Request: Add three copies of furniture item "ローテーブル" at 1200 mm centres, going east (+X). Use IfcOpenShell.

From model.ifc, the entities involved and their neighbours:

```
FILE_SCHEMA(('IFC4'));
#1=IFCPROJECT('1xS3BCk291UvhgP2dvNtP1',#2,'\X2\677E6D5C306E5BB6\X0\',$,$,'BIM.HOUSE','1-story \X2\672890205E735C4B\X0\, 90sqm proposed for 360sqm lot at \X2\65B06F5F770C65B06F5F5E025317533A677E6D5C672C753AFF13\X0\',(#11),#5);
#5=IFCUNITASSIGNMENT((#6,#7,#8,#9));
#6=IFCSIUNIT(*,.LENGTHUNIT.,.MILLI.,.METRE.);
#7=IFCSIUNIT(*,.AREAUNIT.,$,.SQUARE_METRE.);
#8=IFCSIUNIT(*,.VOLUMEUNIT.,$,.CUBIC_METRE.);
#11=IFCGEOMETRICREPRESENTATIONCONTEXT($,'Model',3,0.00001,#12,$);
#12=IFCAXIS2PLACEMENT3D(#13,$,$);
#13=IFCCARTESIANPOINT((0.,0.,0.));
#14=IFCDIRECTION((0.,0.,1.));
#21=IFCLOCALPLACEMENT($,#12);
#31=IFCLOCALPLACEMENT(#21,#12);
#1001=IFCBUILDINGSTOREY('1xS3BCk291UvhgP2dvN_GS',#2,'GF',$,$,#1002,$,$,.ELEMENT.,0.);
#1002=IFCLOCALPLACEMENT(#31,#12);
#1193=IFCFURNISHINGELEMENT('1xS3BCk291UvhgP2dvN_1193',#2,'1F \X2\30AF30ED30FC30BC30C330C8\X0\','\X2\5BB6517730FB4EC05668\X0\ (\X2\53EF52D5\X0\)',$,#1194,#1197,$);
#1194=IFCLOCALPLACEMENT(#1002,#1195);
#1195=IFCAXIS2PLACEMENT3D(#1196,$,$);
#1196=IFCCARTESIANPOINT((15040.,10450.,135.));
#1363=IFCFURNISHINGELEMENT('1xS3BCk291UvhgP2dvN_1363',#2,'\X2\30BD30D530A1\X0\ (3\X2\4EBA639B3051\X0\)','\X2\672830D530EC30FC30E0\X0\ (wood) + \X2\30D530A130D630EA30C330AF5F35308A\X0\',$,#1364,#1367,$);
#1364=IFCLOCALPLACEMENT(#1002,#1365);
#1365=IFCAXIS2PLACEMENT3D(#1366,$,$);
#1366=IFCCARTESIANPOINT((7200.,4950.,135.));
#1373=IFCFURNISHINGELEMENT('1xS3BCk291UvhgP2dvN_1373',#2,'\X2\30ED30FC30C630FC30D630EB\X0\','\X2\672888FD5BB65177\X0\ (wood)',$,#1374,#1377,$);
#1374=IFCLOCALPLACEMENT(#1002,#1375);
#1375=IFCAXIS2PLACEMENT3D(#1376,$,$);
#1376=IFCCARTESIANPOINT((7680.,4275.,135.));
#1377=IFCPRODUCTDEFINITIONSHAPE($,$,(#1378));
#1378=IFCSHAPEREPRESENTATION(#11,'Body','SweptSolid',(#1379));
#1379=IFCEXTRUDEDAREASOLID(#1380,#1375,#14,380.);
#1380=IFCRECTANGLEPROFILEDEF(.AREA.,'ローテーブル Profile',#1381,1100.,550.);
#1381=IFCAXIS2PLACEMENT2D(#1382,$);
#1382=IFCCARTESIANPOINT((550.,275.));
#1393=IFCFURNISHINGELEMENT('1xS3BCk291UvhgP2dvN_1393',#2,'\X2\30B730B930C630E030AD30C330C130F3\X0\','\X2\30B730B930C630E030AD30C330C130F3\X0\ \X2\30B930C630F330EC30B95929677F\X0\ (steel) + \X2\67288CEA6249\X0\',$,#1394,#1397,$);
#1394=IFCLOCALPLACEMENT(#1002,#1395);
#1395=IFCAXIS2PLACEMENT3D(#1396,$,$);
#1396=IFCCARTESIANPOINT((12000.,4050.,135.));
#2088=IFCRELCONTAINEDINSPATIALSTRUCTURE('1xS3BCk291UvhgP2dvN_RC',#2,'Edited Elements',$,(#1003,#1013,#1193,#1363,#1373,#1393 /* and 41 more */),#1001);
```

```python
import numpy as np
import ifcopenshell
import ifcopenshell.api.geometry
import ifcopenshell.api.root
import ifcopenshell.util.element
import ifcopenshell.util.placement
import ifcopenshell.util.unit

model = ifcopenshell.open("model.ifc")
unit_scale = ifcopenshell.util.unit.calculate_unit_scale(model)


def reuse_history(source, copy):
    """copy_class also copies each property set's owner history, people and application; keep the originals."""
    for rel in copy.IsDefinedBy:
        if rel.is_a("IfcRelDefinesByProperties") and (history := rel.RelatingPropertyDefinition.OwnerHistory):
            rel.RelatingPropertyDefinition.OwnerHistory = source.OwnerHistory
            ifcopenshell.util.element.remove_deep2(model, history)


source = model.by_guid("1xS3BCk291UvhgP2dvN_1373")
base = ifcopenshell.util.placement.get_local_placement(source.ObjectPlacement)
step = np.array([1.0, 0.0, 0.0]) * 1.2 / unit_scale

for i in range(1, 4):
    copy = ifcopenshell.api.root.copy_class(model, product=source)
    copy.Representation = ifcopenshell.util.element.copy_deep(
        model, source.Representation, exclude=["IfcGeometricRepresentationContext", "IfcRepresentationMap"]
    )
    reuse_history(source, copy)
    matrix = base.copy()
    matrix[:3, 3] += i * step
    print("added at", matrix[:3, 3].round(3) + 0.0)
    ifcopenshell.api.geometry.edit_object_placement(model, product=copy, matrix=matrix, is_si=False)

model.write("model_v2.ifc")
```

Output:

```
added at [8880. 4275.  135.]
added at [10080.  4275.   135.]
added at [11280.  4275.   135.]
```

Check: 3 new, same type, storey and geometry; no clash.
